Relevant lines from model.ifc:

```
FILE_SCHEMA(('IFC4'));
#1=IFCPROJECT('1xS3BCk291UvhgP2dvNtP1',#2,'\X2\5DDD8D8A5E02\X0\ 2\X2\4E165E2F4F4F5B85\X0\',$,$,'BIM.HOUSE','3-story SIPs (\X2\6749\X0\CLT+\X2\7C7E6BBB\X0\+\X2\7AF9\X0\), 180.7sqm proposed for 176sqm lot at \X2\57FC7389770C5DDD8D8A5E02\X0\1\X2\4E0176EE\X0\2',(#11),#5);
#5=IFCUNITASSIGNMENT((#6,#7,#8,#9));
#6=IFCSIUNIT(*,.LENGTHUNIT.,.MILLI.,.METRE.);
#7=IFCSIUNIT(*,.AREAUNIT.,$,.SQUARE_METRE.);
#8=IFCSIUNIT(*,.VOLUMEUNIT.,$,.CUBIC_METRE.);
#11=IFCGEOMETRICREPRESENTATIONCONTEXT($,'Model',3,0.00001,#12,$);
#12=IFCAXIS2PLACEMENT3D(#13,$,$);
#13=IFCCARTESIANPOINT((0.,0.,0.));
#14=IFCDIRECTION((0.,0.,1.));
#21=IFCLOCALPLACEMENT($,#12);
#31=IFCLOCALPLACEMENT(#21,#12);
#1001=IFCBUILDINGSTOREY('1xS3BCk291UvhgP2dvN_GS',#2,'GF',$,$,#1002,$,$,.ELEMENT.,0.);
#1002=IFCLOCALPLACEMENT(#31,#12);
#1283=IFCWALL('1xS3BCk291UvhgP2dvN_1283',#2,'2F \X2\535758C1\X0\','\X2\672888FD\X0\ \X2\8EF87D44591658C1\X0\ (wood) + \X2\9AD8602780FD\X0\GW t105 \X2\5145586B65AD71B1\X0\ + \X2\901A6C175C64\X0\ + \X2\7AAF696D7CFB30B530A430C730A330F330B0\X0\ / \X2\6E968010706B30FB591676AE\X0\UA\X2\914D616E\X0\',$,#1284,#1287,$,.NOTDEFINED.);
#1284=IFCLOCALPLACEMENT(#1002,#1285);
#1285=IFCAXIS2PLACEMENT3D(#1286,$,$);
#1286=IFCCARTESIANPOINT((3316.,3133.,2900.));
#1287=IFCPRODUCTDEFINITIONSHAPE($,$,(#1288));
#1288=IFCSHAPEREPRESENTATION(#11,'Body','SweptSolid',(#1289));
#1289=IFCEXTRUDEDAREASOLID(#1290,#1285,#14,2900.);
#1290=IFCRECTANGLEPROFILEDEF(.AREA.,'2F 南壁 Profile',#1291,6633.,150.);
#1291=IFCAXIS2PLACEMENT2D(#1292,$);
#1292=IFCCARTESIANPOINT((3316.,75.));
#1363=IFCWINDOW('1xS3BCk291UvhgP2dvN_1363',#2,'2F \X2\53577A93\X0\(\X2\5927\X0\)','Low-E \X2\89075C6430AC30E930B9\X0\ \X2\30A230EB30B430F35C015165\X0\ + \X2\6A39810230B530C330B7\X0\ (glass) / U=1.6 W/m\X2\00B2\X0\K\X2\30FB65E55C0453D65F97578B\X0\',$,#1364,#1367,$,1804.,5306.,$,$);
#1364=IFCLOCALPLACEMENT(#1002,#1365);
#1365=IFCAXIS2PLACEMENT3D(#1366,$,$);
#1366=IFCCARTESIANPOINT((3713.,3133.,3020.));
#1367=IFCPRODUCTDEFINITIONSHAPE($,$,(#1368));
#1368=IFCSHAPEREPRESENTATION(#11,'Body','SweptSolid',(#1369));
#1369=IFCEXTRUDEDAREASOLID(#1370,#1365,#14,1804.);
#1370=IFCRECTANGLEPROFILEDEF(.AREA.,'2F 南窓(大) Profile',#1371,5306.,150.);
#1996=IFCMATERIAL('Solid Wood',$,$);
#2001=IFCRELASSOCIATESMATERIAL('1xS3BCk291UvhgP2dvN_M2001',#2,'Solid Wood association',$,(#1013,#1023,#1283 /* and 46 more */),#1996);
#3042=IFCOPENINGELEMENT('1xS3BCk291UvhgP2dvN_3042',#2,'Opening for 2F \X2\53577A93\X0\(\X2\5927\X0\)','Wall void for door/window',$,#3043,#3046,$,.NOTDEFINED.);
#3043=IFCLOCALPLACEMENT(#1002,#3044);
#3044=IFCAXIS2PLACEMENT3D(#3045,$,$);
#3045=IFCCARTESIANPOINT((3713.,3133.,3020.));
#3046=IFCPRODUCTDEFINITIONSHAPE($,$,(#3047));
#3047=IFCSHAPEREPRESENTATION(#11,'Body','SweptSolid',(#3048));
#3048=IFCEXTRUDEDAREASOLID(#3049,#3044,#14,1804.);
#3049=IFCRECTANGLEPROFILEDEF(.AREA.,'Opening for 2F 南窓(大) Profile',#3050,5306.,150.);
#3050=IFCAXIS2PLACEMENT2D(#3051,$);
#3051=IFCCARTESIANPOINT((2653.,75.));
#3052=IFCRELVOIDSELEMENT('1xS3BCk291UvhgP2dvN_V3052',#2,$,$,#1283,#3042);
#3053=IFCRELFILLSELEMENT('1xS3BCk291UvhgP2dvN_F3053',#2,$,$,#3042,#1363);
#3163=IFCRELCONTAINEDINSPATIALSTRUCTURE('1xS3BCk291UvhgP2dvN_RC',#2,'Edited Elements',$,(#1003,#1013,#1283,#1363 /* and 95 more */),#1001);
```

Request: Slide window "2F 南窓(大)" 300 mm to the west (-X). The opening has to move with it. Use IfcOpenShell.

```python
import ifcopenshell
import ifcopenshell.api.geometry
import ifcopenshell.util.placement

model = ifcopenshell.open("model.ifc")

window = model.by_guid("1xS3BCk291UvhgP2dvN_1363")
opening = window.FillsVoids[0].RelatingOpeningElement
wall = opening.VoidsElements[0].RelatingBuildingElement

wall_matrix = ifcopenshell.util.placement.get_local_placement(wall.ObjectPlacement)
shift = wall_matrix[:3, 0] * -300.0
before = ifcopenshell.util.placement.get_local_placement(window.ObjectPlacement)[:3, 3].copy()

# The window is not placed relative to its opening, so move both.
for product in (opening, window):
    matrix = ifcopenshell.util.placement.get_local_placement(product.ObjectPlacement)
    matrix[:3, 3] += shift
    ifcopenshell.api.geometry.edit_object_placement(model, product=product, matrix=matrix, is_si=False)

after = ifcopenshell.util.placement.get_local_placement(window.ObjectPlacement)[:3, 3]
print("window moved by", (after - before).round(3) + 0.0)

model.write("model_rev.ifc")
```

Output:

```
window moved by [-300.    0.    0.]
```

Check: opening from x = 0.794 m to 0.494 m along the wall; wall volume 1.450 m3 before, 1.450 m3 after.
